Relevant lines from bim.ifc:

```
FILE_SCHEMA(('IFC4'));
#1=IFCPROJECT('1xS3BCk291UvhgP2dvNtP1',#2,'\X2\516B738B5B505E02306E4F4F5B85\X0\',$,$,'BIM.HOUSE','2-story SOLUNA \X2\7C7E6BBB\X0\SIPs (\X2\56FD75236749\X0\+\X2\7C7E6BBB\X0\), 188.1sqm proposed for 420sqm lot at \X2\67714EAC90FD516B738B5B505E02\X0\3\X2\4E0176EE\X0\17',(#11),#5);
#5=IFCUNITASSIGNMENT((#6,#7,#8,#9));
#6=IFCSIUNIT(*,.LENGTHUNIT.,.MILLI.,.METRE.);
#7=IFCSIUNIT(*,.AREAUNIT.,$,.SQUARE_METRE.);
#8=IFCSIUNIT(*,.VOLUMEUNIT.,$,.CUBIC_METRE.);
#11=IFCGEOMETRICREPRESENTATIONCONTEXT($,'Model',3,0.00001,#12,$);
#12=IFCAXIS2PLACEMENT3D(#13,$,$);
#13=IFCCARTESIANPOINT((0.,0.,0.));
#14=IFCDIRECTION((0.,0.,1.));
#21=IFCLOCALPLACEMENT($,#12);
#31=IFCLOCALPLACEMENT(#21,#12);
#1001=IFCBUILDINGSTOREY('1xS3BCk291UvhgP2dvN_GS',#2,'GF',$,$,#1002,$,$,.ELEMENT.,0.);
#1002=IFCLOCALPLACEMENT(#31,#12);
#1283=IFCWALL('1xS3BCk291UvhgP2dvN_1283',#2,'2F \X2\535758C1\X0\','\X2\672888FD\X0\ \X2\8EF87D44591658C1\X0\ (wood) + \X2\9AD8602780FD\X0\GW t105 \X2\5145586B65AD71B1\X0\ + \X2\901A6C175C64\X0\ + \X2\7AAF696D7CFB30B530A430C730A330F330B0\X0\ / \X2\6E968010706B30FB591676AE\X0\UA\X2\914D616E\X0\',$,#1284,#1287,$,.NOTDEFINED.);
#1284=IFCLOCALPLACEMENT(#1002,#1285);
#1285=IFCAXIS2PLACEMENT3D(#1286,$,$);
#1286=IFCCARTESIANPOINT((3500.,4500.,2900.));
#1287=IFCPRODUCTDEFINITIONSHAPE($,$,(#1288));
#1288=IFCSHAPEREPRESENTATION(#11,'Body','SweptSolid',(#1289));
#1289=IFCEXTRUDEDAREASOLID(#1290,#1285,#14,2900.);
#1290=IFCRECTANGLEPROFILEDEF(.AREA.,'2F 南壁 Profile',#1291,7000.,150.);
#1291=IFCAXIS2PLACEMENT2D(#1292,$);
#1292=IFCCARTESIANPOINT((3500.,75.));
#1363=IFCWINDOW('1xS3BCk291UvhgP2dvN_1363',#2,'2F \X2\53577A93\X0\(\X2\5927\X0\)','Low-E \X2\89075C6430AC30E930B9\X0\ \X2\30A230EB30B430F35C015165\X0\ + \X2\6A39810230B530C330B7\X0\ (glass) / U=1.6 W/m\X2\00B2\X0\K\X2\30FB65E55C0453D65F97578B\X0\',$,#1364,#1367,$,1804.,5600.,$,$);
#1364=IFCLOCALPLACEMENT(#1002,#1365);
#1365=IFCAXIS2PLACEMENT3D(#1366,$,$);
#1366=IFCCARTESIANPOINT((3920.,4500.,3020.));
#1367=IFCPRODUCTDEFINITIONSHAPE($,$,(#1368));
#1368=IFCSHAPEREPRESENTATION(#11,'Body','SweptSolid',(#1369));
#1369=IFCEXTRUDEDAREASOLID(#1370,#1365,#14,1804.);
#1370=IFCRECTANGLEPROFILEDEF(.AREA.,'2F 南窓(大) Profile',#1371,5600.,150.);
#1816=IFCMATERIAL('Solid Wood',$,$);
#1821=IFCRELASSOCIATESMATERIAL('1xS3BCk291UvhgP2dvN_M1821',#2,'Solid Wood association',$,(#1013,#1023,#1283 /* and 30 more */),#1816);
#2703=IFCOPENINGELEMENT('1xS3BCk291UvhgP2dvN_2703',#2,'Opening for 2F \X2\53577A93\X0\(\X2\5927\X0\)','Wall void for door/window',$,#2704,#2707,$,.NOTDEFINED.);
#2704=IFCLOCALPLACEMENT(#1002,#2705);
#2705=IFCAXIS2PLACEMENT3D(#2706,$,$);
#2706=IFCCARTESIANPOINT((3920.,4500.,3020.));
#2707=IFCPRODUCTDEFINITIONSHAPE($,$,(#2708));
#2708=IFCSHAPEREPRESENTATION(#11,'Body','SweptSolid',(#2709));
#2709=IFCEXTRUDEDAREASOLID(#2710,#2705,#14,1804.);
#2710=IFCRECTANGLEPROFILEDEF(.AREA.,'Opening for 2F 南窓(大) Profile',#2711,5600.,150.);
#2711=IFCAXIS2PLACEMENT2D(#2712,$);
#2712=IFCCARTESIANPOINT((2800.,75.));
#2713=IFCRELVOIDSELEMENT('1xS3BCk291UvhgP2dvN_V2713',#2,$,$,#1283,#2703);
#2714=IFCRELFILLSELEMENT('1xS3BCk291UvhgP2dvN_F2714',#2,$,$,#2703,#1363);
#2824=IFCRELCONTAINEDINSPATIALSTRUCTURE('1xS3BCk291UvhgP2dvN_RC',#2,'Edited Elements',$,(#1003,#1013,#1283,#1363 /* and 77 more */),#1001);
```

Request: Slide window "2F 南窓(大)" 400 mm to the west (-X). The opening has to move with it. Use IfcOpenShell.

```python
import ifcopenshell
import ifcopenshell.api.geometry
import ifcopenshell.util.placement

model = ifcopenshell.open("bim.ifc")

window = model.by_guid("1xS3BCk291UvhgP2dvN_1363")
opening = window.FillsVoids[0].RelatingOpeningElement
wall = opening.VoidsElements[0].RelatingBuildingElement

wall_matrix = ifcopenshell.util.placement.get_local_placement(wall.ObjectPlacement)
shift = wall_matrix[:3, 0] * -400.0
before = ifcopenshell.util.placement.get_local_placement(window.ObjectPlacement)[:3, 3].copy()

# The window is not placed relative to its opening, so move both.
for product in (opening, window):
    matrix = ifcopenshell.util.placement.get_local_placement(product.ObjectPlacement)
    matrix[:3, 3] += shift
    ifcopenshell.api.geometry.edit_object_placement(model, product=product, matrix=matrix, is_si=False)

after = ifcopenshell.util.placement.get_local_placement(window.ObjectPlacement)[:3, 3]
print("window moved by", (after - before).round(3) + 0.0)

model.write("bim_updated.ifc")
```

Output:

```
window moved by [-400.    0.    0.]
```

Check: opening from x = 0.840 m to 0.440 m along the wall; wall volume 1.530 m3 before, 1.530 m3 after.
